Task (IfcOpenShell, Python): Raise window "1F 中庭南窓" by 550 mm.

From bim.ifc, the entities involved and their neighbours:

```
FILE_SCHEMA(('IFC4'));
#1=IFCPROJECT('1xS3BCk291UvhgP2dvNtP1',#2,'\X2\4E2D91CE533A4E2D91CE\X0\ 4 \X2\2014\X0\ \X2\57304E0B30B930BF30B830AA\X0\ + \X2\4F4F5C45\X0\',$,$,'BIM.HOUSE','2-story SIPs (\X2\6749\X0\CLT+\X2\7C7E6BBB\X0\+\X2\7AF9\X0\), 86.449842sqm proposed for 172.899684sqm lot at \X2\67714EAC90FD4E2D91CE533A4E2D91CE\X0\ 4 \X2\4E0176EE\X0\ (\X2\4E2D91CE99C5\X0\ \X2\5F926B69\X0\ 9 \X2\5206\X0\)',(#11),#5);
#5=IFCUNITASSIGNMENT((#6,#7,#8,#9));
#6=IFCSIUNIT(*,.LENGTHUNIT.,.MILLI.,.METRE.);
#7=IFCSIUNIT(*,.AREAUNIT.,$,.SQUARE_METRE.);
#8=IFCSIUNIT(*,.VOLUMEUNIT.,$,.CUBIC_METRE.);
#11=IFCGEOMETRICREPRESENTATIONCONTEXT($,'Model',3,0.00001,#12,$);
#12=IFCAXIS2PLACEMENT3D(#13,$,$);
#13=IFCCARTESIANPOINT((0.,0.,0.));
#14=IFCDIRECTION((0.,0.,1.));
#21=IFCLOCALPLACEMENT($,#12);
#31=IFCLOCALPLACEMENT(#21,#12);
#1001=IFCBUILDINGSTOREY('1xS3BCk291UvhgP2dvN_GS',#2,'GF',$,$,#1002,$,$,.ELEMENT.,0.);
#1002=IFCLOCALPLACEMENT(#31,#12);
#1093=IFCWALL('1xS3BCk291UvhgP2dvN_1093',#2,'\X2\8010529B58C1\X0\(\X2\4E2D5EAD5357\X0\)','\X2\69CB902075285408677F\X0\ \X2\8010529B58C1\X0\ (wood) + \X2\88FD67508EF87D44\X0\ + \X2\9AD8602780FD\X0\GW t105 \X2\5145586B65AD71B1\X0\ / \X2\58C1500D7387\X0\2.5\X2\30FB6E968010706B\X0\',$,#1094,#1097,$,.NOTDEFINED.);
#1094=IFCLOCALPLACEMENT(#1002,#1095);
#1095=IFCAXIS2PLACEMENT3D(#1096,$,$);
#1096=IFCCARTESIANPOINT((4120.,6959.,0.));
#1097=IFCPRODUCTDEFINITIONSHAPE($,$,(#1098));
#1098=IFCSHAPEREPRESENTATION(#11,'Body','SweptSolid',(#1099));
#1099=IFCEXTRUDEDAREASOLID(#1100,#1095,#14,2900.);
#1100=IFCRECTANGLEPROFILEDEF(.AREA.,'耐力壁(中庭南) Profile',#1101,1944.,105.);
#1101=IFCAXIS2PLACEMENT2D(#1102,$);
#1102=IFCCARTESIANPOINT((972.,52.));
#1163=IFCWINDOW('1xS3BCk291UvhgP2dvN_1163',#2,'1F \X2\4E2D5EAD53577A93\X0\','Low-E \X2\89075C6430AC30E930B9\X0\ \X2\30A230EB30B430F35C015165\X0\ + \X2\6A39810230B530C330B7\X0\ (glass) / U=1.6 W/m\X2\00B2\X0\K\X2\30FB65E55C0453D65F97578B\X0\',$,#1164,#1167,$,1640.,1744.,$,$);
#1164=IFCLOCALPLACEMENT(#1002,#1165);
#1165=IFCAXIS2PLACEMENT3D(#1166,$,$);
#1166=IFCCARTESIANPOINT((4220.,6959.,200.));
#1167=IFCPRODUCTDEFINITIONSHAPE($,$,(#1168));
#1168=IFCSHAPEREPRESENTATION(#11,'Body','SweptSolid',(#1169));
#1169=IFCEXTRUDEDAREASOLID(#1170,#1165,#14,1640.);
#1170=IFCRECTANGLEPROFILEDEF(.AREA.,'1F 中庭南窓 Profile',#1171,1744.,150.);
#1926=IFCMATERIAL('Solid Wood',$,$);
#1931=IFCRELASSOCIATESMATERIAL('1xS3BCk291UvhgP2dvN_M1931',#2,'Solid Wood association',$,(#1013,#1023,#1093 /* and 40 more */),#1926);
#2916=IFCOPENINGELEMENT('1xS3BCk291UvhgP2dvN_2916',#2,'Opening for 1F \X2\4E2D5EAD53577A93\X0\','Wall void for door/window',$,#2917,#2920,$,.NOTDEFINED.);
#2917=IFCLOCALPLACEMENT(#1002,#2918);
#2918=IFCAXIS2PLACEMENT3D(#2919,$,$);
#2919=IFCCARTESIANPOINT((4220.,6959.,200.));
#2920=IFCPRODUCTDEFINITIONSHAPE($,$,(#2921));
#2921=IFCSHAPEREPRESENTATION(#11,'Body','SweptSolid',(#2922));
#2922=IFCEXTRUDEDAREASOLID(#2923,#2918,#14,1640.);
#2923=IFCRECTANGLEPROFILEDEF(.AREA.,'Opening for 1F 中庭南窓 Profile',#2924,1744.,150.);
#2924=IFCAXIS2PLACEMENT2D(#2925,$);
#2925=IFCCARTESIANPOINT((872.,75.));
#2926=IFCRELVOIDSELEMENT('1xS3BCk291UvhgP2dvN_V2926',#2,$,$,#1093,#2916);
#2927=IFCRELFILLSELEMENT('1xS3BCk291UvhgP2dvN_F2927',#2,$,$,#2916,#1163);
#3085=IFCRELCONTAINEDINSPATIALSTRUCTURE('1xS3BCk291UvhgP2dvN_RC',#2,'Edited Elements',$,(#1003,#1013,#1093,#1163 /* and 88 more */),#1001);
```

```python
import numpy as np
import ifcopenshell
import ifcopenshell.api.geometry
import ifcopenshell.util.placement
import ifcopenshell.util.unit

model = ifcopenshell.open("bim.ifc")
unit_scale = ifcopenshell.util.unit.calculate_unit_scale(model)

window = model.by_guid("1xS3BCk291UvhgP2dvN_1163")
opening = window.FillsVoids[0].RelatingOpeningElement
dz = 550.0

shift = np.array([0.0, 0.0, dz])
# The window is not placed relative to its opening, so move both.
for product in (opening, window):
    matrix = ifcopenshell.util.placement.get_local_placement(product.ObjectPlacement)
    matrix[:3, 3] += shift
    ifcopenshell.api.geometry.edit_object_placement(model, product=product, matrix=matrix, is_si=False)

print(f"moved by {dz * unit_scale:+.3f} m")

model.write("bim_rev.ifc")
```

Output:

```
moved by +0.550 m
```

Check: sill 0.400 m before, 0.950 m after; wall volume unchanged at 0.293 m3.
